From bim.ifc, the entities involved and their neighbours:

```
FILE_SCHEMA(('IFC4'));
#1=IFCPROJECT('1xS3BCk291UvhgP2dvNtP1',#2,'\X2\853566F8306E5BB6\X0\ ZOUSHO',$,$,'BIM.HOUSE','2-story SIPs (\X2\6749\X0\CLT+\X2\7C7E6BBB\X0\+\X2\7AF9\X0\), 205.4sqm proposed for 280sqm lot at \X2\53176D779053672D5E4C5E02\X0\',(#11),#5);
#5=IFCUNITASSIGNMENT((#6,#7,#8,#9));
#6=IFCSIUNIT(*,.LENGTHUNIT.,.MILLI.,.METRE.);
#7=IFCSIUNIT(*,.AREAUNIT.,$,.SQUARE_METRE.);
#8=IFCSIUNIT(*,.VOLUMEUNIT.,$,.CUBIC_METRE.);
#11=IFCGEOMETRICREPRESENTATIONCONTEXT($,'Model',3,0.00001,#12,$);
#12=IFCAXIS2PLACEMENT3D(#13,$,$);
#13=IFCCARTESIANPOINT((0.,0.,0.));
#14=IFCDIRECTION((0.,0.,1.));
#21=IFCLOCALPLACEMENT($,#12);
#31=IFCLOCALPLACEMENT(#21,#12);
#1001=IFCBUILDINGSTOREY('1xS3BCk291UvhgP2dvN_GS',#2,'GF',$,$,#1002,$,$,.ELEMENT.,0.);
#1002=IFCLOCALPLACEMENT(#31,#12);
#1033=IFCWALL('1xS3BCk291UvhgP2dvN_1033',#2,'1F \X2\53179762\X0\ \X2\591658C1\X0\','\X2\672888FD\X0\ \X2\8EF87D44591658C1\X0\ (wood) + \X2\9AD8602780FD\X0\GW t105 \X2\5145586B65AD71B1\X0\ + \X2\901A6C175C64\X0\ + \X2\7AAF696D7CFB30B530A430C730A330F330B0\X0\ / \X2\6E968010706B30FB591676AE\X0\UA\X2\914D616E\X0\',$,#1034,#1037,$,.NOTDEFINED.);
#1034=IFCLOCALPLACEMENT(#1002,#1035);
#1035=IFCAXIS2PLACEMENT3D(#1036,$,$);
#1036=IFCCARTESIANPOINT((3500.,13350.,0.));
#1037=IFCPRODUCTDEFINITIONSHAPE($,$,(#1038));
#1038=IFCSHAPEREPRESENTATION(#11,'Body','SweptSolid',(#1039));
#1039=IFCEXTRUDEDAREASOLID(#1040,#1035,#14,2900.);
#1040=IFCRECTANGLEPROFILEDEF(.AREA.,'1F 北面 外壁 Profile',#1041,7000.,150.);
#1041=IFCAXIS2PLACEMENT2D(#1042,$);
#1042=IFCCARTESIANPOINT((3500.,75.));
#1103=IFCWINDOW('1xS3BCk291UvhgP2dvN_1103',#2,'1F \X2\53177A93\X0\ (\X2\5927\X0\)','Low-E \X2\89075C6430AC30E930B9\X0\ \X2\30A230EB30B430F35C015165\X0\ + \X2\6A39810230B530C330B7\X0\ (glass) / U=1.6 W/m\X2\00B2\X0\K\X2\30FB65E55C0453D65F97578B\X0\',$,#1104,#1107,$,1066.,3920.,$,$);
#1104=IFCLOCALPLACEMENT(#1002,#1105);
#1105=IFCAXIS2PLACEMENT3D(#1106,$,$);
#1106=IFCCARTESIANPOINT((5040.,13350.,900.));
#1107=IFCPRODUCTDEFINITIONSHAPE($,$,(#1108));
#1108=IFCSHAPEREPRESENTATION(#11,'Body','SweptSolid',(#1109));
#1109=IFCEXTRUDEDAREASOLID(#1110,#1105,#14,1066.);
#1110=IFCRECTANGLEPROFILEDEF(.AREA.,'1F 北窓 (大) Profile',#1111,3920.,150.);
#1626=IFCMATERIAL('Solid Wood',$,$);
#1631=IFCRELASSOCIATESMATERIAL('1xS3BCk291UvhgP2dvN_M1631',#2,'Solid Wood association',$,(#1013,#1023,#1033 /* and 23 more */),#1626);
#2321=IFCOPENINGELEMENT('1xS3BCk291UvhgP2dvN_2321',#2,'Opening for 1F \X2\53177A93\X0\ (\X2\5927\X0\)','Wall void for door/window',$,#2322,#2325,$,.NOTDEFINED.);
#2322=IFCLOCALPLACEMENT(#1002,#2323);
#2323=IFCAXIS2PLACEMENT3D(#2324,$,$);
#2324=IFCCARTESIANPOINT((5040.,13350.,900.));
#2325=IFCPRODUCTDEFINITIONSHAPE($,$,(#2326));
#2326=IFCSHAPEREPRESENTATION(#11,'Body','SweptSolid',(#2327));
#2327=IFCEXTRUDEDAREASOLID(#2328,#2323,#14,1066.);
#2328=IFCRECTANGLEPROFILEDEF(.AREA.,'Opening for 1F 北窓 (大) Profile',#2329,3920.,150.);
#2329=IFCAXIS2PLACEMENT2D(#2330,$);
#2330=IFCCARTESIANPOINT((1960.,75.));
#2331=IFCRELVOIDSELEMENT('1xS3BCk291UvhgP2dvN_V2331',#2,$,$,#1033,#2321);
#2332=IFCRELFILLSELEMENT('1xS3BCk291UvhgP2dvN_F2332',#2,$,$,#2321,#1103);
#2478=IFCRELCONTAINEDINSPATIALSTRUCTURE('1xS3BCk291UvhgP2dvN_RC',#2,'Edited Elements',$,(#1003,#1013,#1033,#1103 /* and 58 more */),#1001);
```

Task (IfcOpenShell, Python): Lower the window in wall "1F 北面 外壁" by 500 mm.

```python
import numpy as np
import ifcopenshell
import ifcopenshell.api.geometry
import ifcopenshell.util.placement
import ifcopenshell.util.unit

model = ifcopenshell.open("bim.ifc")
unit_scale = ifcopenshell.util.unit.calculate_unit_scale(model)

window = model.by_id(1103)
opening = window.FillsVoids[0].RelatingOpeningElement
dz = -0.5 / unit_scale

shift = np.array([0.0, 0.0, dz])
# The window is not placed relative to its opening, so move both.
for product in (opening, window):
    matrix = ifcopenshell.util.placement.get_local_placement(product.ObjectPlacement)
    matrix[:3, 3] += shift
    ifcopenshell.api.geometry.edit_object_placement(model, product=product, matrix=matrix, is_si=False)

print(f"moved by {dz * unit_scale:+.3f} m")

model.write("bim_rev.ifc")
```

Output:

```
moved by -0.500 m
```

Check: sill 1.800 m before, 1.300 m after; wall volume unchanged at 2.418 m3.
